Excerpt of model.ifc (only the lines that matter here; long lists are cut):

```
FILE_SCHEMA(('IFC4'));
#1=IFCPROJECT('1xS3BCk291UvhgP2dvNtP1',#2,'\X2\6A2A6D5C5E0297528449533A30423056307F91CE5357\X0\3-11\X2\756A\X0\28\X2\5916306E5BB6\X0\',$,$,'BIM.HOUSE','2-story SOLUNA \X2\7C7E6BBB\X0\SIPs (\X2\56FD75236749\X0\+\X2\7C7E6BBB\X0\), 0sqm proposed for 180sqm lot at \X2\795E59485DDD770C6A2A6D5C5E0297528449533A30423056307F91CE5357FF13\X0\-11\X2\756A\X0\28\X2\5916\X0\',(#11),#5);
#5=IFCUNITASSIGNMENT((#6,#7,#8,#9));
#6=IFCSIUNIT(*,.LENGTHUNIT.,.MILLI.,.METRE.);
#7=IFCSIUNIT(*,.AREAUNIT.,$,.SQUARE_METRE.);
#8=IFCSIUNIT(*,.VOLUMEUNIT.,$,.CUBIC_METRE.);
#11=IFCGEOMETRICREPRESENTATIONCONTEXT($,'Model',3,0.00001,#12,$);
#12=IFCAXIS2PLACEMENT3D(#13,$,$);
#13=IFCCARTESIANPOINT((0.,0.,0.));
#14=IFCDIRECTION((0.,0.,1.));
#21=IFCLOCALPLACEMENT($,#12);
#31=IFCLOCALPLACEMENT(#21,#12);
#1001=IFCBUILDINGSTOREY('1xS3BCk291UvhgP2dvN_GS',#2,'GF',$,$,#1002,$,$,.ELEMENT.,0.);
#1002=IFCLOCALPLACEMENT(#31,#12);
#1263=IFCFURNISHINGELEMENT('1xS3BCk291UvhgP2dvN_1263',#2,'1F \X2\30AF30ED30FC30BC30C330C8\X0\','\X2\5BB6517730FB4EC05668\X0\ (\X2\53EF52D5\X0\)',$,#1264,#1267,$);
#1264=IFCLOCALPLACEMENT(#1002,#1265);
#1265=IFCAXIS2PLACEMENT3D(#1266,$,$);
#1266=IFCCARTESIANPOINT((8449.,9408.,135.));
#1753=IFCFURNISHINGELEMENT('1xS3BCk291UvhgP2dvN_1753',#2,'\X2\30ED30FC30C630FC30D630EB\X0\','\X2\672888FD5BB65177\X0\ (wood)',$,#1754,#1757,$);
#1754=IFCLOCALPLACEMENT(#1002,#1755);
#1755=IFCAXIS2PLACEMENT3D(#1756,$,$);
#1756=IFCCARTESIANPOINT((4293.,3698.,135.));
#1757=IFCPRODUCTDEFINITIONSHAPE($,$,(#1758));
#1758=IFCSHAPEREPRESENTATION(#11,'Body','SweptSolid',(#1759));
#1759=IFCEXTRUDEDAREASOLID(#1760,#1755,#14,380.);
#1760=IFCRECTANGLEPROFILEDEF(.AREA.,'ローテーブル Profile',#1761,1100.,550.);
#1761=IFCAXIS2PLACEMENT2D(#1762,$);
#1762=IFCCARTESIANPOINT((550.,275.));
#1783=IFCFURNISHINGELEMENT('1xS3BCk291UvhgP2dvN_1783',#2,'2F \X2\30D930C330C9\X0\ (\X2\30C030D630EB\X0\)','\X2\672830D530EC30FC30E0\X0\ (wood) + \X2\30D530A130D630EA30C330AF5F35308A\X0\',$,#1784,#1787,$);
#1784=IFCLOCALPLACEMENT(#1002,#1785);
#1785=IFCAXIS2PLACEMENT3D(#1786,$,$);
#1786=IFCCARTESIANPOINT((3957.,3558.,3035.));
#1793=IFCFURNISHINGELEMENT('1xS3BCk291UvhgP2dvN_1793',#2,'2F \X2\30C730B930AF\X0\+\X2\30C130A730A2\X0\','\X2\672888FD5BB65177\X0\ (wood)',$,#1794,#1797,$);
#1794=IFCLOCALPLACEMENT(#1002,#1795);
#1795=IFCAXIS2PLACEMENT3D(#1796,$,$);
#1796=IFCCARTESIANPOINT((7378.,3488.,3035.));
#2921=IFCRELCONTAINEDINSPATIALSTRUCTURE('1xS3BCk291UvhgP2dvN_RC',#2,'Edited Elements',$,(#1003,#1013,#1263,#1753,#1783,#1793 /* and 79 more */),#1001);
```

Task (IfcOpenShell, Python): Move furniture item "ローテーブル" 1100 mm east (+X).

```python
import ifcopenshell
import ifcopenshell.api.geometry
import ifcopenshell.util.placement
import ifcopenshell.util.unit

model = ifcopenshell.open("model.ifc")
unit_scale = ifcopenshell.util.unit.calculate_unit_scale(model)

item = model.by_guid("1xS3BCk291UvhgP2dvN_1753")
matrix = ifcopenshell.util.placement.get_local_placement(item.ObjectPlacement)
matrix[0, 3] += 1.1 / unit_scale
ifcopenshell.api.geometry.edit_object_placement(model, product=item, matrix=matrix, is_si=False)

print(ifcopenshell.util.placement.get_local_placement(item.ObjectPlacement).round(3) + 0.0)

model.write("model_rev.ifc")
```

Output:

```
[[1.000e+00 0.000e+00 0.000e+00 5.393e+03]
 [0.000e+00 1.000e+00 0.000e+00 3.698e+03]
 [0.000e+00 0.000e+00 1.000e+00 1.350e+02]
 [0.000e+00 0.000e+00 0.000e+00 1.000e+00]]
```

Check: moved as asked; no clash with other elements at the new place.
